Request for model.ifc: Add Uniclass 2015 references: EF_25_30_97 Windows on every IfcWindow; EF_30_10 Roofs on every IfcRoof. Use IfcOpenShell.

First a look at what the model holds.

```python
import ifcopenshell

model = ifcopenshell.open("model.ifc")
print(model.schema)
print("classifications:", [c.Name for c in model.by_type("IfcClassification")])
for ifc_class in ("IfcDoor", "IfcRoof", "IfcStair", "IfcWall", "IfcWindow"):
    print(ifc_class, len(model.by_type(ifc_class)))
```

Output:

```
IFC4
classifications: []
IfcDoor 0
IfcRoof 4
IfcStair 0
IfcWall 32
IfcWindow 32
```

```python
import ifcopenshell
import ifcopenshell.api.classification

model = ifcopenshell.open("model.ifc")

system = ifcopenshell.api.classification.add_classification(model, classification="Uniclass 2015")

codes = {
    "IfcWindow": ("EF_25_30_97", "Windows"),
    "IfcRoof": ("EF_30_10", "Roofs"),
}
for ifc_class, (code, name) in codes.items():
    products = model.by_type(ifc_class)
    ifcopenshell.api.classification.add_reference(
        model, products=products, classification=system, identification=code, name=name
    )
    print(code, len(products))

model.write("model_updated.ifc")
```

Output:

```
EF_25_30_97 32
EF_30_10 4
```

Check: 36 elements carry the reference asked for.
